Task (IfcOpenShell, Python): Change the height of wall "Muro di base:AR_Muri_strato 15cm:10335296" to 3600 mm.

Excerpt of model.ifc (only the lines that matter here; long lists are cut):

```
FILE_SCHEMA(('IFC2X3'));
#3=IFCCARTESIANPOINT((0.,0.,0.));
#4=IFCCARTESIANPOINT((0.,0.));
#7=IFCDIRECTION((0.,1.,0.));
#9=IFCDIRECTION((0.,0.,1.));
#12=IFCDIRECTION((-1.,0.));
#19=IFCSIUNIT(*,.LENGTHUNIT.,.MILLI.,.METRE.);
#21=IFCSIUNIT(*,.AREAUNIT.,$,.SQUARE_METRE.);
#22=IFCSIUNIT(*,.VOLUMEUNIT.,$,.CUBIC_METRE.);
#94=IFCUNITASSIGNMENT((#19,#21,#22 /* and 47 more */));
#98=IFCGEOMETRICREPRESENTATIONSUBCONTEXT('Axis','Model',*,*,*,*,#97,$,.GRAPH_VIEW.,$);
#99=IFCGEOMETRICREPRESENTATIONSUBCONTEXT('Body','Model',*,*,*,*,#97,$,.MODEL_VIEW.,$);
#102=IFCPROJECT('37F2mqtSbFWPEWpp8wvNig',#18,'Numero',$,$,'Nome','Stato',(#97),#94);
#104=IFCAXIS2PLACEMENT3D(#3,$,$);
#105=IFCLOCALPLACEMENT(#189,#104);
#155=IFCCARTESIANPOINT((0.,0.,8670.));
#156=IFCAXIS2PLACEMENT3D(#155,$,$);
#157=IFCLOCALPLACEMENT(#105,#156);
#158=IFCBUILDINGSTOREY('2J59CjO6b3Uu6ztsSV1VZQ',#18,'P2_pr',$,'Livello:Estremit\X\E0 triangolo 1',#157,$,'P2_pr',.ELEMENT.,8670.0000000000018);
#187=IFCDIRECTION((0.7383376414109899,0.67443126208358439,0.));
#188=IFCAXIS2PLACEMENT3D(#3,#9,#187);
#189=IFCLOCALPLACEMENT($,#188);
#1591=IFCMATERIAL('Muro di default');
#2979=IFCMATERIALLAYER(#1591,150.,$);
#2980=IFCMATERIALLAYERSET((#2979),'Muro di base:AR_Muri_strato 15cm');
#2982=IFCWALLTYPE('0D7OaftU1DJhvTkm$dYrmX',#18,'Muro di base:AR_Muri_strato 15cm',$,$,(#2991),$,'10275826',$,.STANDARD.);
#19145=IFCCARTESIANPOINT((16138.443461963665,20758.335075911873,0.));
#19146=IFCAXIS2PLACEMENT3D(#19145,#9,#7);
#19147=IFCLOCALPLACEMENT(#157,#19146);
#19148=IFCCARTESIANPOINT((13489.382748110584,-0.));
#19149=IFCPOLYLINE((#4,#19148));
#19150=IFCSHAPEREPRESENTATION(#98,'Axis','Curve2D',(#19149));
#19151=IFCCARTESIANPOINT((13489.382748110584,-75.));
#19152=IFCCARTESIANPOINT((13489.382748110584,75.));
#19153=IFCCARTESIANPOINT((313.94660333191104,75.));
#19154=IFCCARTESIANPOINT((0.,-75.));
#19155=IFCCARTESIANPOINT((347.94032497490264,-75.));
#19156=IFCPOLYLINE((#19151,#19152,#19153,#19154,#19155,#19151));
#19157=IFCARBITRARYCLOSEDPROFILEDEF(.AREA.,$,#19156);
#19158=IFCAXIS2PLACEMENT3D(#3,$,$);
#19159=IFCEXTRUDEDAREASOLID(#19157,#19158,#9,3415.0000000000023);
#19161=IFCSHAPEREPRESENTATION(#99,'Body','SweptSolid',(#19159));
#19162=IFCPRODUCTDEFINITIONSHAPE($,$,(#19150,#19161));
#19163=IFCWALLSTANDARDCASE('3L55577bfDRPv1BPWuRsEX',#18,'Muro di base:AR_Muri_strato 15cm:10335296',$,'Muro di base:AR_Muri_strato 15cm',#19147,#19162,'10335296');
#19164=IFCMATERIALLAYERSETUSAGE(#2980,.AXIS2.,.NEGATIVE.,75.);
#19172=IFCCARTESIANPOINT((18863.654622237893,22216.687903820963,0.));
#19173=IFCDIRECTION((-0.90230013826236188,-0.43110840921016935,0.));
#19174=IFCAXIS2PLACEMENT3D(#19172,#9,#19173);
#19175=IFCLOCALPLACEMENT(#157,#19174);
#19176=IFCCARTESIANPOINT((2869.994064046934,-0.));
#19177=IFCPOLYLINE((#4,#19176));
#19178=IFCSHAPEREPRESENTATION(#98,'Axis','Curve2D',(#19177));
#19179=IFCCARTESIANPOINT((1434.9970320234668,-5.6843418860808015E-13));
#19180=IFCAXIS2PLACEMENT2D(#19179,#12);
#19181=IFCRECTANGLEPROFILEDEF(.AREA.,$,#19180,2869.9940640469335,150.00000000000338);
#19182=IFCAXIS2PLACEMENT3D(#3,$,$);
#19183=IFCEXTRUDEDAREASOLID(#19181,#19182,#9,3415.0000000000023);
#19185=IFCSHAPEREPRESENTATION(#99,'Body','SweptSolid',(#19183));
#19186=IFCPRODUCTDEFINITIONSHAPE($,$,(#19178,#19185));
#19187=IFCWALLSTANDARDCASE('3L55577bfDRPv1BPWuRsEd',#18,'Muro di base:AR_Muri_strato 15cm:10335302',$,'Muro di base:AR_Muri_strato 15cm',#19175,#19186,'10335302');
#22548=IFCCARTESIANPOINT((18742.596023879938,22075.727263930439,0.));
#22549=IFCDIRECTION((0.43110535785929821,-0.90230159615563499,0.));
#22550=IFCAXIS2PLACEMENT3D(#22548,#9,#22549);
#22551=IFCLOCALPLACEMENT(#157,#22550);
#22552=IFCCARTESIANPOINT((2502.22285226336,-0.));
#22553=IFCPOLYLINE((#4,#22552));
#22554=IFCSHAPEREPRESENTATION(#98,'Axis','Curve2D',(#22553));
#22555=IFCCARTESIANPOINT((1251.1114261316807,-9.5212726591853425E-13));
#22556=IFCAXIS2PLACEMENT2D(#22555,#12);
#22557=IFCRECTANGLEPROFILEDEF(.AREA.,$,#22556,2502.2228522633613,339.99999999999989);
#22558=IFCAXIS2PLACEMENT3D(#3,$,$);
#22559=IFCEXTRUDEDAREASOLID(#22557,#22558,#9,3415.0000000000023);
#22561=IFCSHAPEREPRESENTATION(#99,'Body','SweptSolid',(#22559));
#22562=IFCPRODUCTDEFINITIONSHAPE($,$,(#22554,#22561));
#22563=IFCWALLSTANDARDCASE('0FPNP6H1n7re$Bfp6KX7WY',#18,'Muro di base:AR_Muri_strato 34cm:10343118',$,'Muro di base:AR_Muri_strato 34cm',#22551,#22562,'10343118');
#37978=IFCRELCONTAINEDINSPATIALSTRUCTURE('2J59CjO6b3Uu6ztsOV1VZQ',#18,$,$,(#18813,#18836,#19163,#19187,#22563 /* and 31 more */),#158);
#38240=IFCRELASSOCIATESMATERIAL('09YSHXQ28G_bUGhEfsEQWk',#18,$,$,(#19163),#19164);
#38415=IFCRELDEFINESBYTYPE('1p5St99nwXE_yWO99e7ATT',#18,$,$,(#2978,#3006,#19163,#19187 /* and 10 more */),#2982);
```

```python
import ifcopenshell
import ifcopenshell.geom
import ifcopenshell.util.representation
import ifcopenshell.util.shape
import ifcopenshell.util.unit

model = ifcopenshell.open("model.ifc")
unit_scale = ifcopenshell.util.unit.calculate_unit_scale(model)
settings = ifcopenshell.geom.settings()


def volume(element):
    """Net volume in cubic metres, openings subtracted."""
    shape = ifcopenshell.geom.create_shape(settings, element)
    return ifcopenshell.util.shape.get_volume(shape.geometry)


wall = model.by_id(19163)
before = volume(wall)

body = ifcopenshell.util.representation.get_representation(wall, "Model", "Body")
solid = body.Items[0]
old_height = solid.Depth
solid.Depth = 3.6 / unit_scale
after = volume(wall)

print(f"height {old_height:g} -> {solid.Depth:g}, volume {before:.3f} -> {after:.3f} m3")

model.write("model_v2.ifc")
```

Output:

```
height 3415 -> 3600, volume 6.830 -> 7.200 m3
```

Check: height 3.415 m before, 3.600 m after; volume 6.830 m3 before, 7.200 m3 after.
